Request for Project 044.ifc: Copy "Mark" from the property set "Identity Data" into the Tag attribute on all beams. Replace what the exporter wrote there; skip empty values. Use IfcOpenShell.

First a look at what the model holds.

```python
import ifcopenshell
import ifcopenshell.util.element

model = ifcopenshell.open("Project 044.ifc")
print(model.schema)
beams = model.by_type("IfcBeam")
print(len(beams), "beams")
for e in beams[:8]:
    source = ifcopenshell.util.element.get_pset(e, "Identity Data", "Mark")
    target = e.Tag
    print(e.id(), repr(source), repr(target), sep=" | ")
```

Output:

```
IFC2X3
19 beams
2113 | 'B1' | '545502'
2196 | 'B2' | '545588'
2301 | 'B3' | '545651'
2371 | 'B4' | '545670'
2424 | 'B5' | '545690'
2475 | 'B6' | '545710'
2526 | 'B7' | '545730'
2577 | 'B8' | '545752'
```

```python
import ifcopenshell
import ifcopenshell.util.element

model = ifcopenshell.open("Project 044.ifc")

count = 0
for e in model.by_type("IfcBeam"):
    value = ifcopenshell.util.element.get_pset(e, "Identity Data", "Mark")
    current = e.Tag
    if not value or not value.strip() or current == value:
        continue
    e.Tag = value
    count += 1

print(count, "beams updated")

model.write("Project 044_v2.ifc")
```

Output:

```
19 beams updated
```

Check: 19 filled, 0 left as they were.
